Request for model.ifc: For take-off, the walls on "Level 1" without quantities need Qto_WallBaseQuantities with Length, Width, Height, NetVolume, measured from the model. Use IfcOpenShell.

First a look at what the model holds.

```python
import ifcopenshell
import ifcopenshell.util.element
import ifcopenshell.util.unit

model = ifcopenshell.open("model.ifc")
print(model.schema)
for unit_type in ("LENGTHUNIT", "AREAUNIT", "VOLUMEUNIT"):
    print(unit_type, ifcopenshell.util.unit.calculate_unit_scale(model, unit_type))
storey = next(s for s in model.by_type("IfcBuildingStorey") if s.Name == "Level 1")
walls = [e for e in ifcopenshell.util.element.get_decomposition(storey) if e.is_a("IfcWall")]
for e in sorted(walls, key=lambda e: e.id()):
    print(e.id(), e.is_a(), e.Name, list(ifcopenshell.util.element.get_psets(e, qtos_only=True)), sep=" | ")
```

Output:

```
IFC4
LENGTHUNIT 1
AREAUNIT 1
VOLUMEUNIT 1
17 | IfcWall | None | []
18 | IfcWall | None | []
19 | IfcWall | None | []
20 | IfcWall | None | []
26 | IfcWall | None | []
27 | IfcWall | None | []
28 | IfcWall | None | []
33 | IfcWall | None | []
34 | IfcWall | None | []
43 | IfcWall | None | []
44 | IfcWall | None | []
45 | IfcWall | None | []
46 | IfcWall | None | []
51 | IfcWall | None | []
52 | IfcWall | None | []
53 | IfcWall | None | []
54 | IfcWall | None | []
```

```python
import ifcopenshell
import ifcopenshell.api.pset
import ifcopenshell.geom
import ifcopenshell.util.element
import ifcopenshell.util.shape
import ifcopenshell.util.unit

model = ifcopenshell.open("model.ifc")
unit_scale = ifcopenshell.util.unit.calculate_unit_scale(model)
volume_scale = ifcopenshell.util.unit.calculate_unit_scale(model, "VOLUMEUNIT")
settings = ifcopenshell.geom.settings()

storey = next(s for s in model.by_type("IfcBuildingStorey") if s.Name == "Level 1")
walls = [e for e in ifcopenshell.util.element.get_decomposition(storey) if e.is_a("IfcWall")]

for e in sorted(walls, key=lambda e: e.id()):
    if ifcopenshell.util.element.get_psets(e, qtos_only=True, should_inherit=False):
        continue
    # Geometry comes back in metres, in the element's own axes.
    shape = ifcopenshell.geom.create_shape(settings, e)
    values = {
        "Length": ifcopenshell.util.shape.get_x(shape.geometry) / unit_scale,
        "Width": ifcopenshell.util.shape.get_y(shape.geometry) / unit_scale,
        "Height": ifcopenshell.util.shape.get_z(shape.geometry) / unit_scale,
        "NetVolume": ifcopenshell.util.shape.get_volume(shape.geometry) / volume_scale,
    }
    qto = ifcopenshell.api.pset.add_qto(model, product=e, name="Qto_WallBaseQuantities")
    ifcopenshell.api.pset.edit_qto(model, qto=qto, properties=values)
    print(e.id(), {k: round(v, 3) for k, v in values.items()})

model.write("model_edited.ifc")
```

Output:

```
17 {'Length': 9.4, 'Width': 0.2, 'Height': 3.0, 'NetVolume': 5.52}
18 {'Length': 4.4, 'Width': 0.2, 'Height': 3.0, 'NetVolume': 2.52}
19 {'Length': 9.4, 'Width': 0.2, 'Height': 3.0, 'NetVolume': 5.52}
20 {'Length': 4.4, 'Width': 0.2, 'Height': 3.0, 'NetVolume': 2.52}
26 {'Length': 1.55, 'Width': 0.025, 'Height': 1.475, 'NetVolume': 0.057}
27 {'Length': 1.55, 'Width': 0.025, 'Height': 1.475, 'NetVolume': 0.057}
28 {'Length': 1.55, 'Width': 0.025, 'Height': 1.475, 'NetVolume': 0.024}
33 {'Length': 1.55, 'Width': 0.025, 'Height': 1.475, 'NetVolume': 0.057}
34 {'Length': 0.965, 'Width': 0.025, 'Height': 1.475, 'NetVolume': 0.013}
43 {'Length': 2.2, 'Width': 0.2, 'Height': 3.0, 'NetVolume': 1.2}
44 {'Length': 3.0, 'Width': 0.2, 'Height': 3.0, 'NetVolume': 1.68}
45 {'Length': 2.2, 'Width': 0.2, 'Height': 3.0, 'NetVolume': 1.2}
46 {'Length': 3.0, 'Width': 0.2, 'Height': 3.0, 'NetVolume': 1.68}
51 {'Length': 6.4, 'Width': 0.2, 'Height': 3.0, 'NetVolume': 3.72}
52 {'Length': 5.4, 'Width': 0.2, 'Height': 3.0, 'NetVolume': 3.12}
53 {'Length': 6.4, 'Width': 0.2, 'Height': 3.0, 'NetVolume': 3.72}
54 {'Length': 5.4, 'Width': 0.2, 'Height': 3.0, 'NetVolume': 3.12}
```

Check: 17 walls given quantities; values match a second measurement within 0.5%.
